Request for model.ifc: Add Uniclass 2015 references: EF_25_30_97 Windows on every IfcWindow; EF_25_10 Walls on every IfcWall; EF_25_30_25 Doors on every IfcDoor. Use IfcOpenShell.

First a look at what the model holds.

```python
import ifcopenshell

model = ifcopenshell.open("model.ifc")
print(model.schema)
print("classifications:", [c.Name for c in model.by_type("IfcClassification")])
for ifc_class in ("IfcDoor", "IfcRoof", "IfcStair", "IfcWall", "IfcWindow"):
    print(ifc_class, len(model.by_type(ifc_class)))
```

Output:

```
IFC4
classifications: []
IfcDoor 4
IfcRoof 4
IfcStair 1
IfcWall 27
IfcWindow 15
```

```python
import ifcopenshell
import ifcopenshell.api.classification

model = ifcopenshell.open("model.ifc")

system = ifcopenshell.api.classification.add_classification(model, classification="Uniclass 2015")

codes = {
    "IfcWindow": ("EF_25_30_97", "Windows"),
    "IfcWall": ("EF_25_10", "Walls"),
    "IfcDoor": ("EF_25_30_25", "Doors"),
}
for ifc_class, (code, name) in codes.items():
    products = model.by_type(ifc_class)
    ifcopenshell.api.classification.add_reference(
        model, products=products, classification=system, identification=code, name=name
    )
    print(code, len(products))

model.write("model-out.ifc")
```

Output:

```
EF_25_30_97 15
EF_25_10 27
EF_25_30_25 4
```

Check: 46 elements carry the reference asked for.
